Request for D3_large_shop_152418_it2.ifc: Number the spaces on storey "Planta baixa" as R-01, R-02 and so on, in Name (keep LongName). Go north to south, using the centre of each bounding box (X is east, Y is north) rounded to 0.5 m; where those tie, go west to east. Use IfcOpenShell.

First a look at what the model holds.

```python
import ifcopenshell
import ifcopenshell.util.element
import ifcopenshell.util.placement

model = ifcopenshell.open("D3_large_shop_152418_it2.ifc")
print(model.schema)
storey = next(s for s in model.by_type("IfcBuildingStorey") if s.Name == "Planta baixa")
spaces = [e for e in ifcopenshell.util.element.get_decomposition(storey) if e.is_a("IfcSpace")]
for e in sorted(spaces, key=lambda e: e.id()):
    origin = ifcopenshell.util.placement.get_local_placement(e.ObjectPlacement)[:3, 3]
    print(e.id(), e.Name, e.LongName, origin.round(2) + 0.0, sep=" | ")
```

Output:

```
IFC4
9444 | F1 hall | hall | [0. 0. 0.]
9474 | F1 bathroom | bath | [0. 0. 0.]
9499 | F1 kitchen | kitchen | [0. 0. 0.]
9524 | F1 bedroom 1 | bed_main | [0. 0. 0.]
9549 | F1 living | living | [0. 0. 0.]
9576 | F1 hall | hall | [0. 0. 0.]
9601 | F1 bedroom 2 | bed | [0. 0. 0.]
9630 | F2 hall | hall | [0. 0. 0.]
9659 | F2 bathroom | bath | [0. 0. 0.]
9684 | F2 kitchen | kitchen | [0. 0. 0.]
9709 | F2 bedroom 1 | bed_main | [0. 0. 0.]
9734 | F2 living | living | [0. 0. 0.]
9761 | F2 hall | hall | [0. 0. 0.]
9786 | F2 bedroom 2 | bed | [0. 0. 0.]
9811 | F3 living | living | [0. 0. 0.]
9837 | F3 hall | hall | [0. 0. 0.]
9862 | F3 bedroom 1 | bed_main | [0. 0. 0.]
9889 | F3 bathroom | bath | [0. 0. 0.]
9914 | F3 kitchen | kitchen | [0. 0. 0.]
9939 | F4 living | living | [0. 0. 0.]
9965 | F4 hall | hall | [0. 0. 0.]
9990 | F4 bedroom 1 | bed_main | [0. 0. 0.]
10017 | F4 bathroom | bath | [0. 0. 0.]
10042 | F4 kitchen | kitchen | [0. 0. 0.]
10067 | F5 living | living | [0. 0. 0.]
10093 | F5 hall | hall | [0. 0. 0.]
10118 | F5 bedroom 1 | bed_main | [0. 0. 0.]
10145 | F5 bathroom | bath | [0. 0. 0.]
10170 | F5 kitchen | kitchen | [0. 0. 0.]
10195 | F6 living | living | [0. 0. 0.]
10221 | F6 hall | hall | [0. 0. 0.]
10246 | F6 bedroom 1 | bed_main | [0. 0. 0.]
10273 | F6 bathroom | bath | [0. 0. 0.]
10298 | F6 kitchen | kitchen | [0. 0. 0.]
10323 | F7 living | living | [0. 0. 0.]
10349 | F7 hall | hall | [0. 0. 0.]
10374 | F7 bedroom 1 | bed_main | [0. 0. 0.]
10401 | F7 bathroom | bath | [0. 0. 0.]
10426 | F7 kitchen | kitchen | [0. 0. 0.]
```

```python
import ifcopenshell
import ifcopenshell.geom
import ifcopenshell.util.element
import ifcopenshell.util.shape

model = ifcopenshell.open("D3_large_shop_152418_it2.ifc")
settings = ifcopenshell.geom.settings()
settings.set("use-world-coords", True)


def centre(element):
    shape = ifcopenshell.geom.create_shape(settings, element)
    return ifcopenshell.util.shape.get_bbox_centroid(shape.geometry)


storey = next(s for s in model.by_type("IfcBuildingStorey") if s.Name == "Planta baixa")
spaces = [e for e in ifcopenshell.util.element.get_decomposition(storey) if e.is_a("IfcSpace")]

# Insertion points can sit at a corner or the storey origin, so sort by the geometry (in metres).
centres = {e: centre(e) for e in spaces}
spaces.sort(key=lambda e: (-round(centres[e][1] / 0.5), centres[e][0]))

for i, e in enumerate(spaces, start=1):
    number = f"R-{i:02d}"
    e.Name = number
    print(e.id(), number)

model.write("D3_large_shop_152418_it2_edited.ifc")
```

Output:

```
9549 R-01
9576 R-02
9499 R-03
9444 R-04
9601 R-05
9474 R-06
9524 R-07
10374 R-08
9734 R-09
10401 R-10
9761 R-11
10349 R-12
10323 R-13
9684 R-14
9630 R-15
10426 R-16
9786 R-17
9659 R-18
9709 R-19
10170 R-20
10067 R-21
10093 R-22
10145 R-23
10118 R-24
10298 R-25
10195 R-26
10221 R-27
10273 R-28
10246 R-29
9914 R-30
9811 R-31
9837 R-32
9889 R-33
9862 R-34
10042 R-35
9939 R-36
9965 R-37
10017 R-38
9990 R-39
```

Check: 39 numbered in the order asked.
